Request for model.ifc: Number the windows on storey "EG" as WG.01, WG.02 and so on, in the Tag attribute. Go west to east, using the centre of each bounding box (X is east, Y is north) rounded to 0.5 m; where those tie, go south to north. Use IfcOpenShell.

First a look at what the model holds.

```python
import ifcopenshell
import ifcopenshell.util.element
import ifcopenshell.util.placement

model = ifcopenshell.open("model.ifc")
print(model.schema)
storey = next(s for s in model.by_type("IfcBuildingStorey") if s.Name == "EG")
windows = [e for e in ifcopenshell.util.element.get_decomposition(storey) if e.is_a("IfcWindow")]
for e in sorted(windows, key=lambda e: e.id()):
    origin = ifcopenshell.util.placement.get_local_placement(e.ObjectPlacement)[:3, 3]
    print(e.id(), e.Tag, e.Name, origin.round(2) + 0.0, sep=" | ")
```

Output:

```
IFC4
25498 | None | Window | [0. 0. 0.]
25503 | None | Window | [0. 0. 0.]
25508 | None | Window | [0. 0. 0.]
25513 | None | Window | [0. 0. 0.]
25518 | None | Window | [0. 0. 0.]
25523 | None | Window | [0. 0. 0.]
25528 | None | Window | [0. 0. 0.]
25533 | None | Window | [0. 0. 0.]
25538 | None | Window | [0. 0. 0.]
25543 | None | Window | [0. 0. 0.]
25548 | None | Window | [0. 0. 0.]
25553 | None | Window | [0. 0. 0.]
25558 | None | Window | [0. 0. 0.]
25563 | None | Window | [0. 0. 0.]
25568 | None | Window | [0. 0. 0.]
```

```python
import ifcopenshell
import ifcopenshell.geom
import ifcopenshell.util.element
import ifcopenshell.util.shape

model = ifcopenshell.open("model.ifc")
settings = ifcopenshell.geom.settings()
settings.set("use-world-coords", True)


def centre(element):
    shape = ifcopenshell.geom.create_shape(settings, element)
    return ifcopenshell.util.shape.get_bbox_centroid(shape.geometry)


storey = next(s for s in model.by_type("IfcBuildingStorey") if s.Name == "EG")
windows = [e for e in ifcopenshell.util.element.get_decomposition(storey) if e.is_a("IfcWindow")]

# Insertion points can sit at a corner or the storey origin, so sort by the geometry (in metres).
centres = {e: centre(e) for e in windows}
windows.sort(key=lambda e: (round(centres[e][0] / 0.5), centres[e][1]))

for i, e in enumerate(windows, start=1):
    number = f"WG.{i:02d}"
    e.Tag = number
    print(e.id(), number)

model.write("model-out.ifc")
```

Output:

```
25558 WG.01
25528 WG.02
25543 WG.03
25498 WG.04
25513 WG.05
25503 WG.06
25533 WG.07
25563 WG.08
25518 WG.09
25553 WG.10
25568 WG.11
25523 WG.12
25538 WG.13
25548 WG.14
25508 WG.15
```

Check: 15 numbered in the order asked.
